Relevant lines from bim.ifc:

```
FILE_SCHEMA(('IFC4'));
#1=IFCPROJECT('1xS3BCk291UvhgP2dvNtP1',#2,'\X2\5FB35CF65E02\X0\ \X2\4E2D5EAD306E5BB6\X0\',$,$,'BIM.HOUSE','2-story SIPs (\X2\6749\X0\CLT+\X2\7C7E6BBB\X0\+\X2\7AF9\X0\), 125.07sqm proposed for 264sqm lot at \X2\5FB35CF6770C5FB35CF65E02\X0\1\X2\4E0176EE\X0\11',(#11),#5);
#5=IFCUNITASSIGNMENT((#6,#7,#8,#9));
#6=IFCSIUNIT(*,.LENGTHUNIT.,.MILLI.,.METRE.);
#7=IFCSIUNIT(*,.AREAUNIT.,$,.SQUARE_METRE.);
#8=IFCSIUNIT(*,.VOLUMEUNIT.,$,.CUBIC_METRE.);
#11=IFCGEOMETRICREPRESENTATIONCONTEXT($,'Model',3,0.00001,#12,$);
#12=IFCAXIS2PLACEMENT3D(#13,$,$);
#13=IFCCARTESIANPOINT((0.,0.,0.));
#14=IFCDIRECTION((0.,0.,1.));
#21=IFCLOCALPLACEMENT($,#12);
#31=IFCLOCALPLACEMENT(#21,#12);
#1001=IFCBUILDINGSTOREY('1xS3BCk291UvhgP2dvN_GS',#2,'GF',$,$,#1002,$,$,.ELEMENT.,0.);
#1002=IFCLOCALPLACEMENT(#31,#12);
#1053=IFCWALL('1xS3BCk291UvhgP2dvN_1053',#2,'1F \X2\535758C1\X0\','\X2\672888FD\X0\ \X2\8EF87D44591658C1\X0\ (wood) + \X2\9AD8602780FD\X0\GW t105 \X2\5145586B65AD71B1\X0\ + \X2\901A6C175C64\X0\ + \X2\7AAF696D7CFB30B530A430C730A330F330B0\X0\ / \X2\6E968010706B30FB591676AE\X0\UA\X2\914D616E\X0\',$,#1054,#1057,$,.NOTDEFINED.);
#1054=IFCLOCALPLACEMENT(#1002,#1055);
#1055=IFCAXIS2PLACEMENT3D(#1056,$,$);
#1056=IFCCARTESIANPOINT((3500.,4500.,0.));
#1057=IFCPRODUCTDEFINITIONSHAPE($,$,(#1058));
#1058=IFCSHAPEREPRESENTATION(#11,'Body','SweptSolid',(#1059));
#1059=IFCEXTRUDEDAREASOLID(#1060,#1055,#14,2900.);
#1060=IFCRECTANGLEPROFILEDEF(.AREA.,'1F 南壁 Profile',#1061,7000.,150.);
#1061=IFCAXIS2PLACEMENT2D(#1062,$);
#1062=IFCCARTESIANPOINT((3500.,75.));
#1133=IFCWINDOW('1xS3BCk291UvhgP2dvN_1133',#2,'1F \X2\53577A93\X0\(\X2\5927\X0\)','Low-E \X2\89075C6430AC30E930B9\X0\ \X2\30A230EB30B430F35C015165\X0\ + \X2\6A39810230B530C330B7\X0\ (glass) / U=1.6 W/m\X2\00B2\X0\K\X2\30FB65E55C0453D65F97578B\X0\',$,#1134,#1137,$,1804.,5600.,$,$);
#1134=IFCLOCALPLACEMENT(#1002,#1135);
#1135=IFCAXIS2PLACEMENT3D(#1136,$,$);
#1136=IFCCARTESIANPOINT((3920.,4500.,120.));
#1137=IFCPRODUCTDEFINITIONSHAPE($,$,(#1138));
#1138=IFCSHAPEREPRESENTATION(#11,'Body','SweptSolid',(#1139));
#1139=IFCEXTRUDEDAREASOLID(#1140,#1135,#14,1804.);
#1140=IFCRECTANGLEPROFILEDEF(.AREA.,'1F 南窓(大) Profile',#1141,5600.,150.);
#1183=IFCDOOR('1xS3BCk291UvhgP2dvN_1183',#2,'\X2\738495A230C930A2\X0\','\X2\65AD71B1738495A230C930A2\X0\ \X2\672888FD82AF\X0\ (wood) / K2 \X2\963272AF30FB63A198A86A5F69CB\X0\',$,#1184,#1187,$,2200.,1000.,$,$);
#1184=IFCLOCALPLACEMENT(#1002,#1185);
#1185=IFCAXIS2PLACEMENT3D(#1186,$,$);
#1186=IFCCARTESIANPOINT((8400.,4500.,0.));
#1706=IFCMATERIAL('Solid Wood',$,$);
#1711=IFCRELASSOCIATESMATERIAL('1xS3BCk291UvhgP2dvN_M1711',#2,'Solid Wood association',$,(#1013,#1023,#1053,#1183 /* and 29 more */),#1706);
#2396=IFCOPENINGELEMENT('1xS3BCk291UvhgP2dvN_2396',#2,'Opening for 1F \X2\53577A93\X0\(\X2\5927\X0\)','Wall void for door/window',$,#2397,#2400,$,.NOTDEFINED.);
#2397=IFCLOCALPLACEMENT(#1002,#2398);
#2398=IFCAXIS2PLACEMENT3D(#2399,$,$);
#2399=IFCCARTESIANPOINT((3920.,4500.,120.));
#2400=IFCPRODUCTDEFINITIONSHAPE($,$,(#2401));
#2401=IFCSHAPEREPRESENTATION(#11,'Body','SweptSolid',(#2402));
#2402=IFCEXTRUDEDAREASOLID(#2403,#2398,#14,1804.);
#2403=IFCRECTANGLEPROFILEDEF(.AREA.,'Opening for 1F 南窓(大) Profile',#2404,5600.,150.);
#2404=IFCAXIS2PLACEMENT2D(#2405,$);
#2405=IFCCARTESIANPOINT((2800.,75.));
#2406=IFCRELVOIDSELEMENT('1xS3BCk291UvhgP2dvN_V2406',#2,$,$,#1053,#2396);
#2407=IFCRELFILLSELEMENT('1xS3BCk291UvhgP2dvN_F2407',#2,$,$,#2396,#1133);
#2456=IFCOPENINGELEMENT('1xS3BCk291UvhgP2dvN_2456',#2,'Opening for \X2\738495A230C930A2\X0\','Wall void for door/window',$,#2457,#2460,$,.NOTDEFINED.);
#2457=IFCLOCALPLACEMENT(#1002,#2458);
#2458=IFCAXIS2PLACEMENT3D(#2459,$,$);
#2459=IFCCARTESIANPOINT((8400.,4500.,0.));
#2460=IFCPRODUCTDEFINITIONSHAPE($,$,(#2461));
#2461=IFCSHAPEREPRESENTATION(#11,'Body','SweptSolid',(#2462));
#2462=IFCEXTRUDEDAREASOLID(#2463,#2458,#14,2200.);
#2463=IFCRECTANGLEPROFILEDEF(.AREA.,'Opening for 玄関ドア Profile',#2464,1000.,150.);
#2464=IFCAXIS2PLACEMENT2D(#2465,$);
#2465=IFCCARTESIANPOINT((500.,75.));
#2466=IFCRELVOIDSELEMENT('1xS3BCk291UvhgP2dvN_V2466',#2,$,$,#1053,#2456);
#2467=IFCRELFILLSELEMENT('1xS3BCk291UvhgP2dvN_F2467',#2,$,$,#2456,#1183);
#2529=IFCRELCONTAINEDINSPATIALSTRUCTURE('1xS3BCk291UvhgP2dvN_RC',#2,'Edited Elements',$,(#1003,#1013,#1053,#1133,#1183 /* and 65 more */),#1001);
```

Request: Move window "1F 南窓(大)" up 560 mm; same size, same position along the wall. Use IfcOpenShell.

```python
import numpy as np
import ifcopenshell
import ifcopenshell.api.geometry
import ifcopenshell.util.placement
import ifcopenshell.util.unit

model = ifcopenshell.open("bim.ifc")
unit_scale = ifcopenshell.util.unit.calculate_unit_scale(model)

window = model.by_guid("1xS3BCk291UvhgP2dvN_1133")
opening = window.FillsVoids[0].RelatingOpeningElement
dz = 0.56 / unit_scale

shift = np.array([0.0, 0.0, dz])
# The window is not placed relative to its opening, so move both.
for product in (opening, window):
    matrix = ifcopenshell.util.placement.get_local_placement(product.ObjectPlacement)
    matrix[:3, 3] += shift
    ifcopenshell.api.geometry.edit_object_placement(model, product=product, matrix=matrix, is_si=False)

print(f"moved by {dz * unit_scale:+.3f} m")

model.write("bim-out.ifc")
```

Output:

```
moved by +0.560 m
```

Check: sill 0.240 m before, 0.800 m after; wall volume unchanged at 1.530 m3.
